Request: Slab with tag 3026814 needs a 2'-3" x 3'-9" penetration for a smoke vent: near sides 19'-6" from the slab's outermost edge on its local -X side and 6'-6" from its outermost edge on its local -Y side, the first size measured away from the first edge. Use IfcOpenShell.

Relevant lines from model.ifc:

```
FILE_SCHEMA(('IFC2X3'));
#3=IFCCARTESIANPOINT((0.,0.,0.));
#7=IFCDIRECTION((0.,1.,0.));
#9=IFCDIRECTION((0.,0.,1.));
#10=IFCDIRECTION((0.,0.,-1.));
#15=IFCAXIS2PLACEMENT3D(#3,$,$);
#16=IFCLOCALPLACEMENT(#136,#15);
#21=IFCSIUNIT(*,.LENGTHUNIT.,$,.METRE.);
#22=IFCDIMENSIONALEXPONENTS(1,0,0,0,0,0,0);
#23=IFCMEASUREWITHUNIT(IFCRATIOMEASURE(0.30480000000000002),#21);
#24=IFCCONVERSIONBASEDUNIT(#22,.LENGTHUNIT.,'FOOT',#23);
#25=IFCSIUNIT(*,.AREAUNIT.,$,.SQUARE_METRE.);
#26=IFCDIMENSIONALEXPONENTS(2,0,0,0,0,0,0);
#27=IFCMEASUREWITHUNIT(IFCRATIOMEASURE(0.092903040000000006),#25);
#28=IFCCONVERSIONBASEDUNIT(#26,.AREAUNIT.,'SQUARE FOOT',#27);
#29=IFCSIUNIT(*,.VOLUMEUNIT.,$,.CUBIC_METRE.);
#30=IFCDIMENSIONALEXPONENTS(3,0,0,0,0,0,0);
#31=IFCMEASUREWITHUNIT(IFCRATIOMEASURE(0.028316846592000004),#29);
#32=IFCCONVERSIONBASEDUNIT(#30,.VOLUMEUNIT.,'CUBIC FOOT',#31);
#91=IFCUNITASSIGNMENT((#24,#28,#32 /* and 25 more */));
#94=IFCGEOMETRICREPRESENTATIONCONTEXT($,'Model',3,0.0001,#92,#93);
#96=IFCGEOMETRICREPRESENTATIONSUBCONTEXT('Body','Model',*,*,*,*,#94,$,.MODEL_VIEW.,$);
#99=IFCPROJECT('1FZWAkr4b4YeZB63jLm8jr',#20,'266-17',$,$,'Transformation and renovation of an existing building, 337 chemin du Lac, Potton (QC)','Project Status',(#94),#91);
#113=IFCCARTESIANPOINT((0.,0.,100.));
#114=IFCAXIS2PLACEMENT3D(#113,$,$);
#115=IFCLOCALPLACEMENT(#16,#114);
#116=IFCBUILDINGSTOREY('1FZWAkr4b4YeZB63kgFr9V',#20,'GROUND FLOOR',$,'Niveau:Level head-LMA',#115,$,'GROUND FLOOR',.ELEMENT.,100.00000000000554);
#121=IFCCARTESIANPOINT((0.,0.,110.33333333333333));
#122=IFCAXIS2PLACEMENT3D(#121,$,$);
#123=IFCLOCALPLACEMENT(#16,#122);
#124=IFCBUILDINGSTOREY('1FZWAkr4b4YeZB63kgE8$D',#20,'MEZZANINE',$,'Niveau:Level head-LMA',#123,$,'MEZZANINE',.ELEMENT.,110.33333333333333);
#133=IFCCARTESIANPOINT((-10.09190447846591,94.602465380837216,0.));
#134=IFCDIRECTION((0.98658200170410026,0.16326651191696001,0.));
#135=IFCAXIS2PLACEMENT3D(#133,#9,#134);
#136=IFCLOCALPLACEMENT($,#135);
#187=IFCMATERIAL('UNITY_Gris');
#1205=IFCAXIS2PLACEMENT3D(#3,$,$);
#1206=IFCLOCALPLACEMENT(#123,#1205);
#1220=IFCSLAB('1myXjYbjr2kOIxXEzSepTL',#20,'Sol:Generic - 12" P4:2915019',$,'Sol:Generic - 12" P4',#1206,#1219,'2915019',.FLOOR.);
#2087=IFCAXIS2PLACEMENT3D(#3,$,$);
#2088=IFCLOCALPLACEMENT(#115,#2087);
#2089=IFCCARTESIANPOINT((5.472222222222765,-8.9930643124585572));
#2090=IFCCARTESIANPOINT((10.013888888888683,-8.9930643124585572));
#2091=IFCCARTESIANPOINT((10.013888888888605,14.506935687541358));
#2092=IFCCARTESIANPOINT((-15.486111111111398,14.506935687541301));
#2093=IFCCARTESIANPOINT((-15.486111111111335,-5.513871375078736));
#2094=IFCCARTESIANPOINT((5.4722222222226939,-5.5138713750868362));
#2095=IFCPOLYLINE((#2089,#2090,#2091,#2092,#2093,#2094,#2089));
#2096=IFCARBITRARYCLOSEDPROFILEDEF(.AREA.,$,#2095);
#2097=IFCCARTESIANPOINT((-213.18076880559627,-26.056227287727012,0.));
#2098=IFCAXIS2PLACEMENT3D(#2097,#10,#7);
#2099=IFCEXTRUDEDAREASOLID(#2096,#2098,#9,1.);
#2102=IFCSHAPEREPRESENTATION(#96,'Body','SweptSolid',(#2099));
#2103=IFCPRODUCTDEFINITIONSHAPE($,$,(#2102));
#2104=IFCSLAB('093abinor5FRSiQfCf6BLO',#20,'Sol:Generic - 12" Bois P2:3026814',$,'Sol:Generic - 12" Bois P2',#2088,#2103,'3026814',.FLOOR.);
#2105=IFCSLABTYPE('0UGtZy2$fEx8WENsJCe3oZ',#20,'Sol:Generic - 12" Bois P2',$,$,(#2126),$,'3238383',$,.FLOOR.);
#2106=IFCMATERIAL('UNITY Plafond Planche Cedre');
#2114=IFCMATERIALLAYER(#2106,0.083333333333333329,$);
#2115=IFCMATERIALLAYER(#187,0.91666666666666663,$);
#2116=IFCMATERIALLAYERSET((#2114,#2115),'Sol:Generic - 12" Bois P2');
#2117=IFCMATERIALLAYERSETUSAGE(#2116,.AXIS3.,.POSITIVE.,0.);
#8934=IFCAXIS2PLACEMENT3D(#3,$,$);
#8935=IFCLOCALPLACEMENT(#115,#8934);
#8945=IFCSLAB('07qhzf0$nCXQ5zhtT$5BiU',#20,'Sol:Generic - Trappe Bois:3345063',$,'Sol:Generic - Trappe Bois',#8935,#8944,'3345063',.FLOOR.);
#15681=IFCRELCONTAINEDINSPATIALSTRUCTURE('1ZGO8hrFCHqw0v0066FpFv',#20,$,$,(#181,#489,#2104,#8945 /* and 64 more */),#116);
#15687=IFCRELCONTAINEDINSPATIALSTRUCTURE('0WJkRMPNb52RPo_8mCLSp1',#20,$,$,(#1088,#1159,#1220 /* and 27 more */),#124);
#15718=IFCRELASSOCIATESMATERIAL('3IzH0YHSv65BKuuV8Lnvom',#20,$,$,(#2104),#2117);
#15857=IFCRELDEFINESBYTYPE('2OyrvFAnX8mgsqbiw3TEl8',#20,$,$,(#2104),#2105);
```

```python
import numpy as np
import ifcopenshell
import ifcopenshell.api.feature
import ifcopenshell.api.geometry
import ifcopenshell.api.root
import ifcopenshell.geom
import ifcopenshell.util.placement
import ifcopenshell.util.representation
import ifcopenshell.util.shape
import ifcopenshell.util.unit

model = ifcopenshell.open("model.ifc")
unit_scale = ifcopenshell.util.unit.calculate_unit_scale(model)
settings = ifcopenshell.geom.settings()


def volume(element):
    """Net volume in cubic metres, openings subtracted."""
    shape = ifcopenshell.geom.create_shape(settings, element)
    return ifcopenshell.util.shape.get_volume(shape.geometry)


slab = model.by_guid("093abinor5FRSiQfCf6BLO")
before = volume(slab)

# Extent in the slab's own axes, in metres. The edges named are its -X and -Y sides.
slab_shape = ifcopenshell.geom.create_shape(settings, slab)
vertices = ifcopenshell.util.shape.get_vertices(slab_shape.geometry)
x_min, y_min, bottom = vertices.min(axis=0)
top = vertices[:, 2].max()

opening = ifcopenshell.api.root.create_entity(model, ifc_class="IfcOpeningElement", name="Smoke vent opening")
context = ifcopenshell.util.representation.get_context(model, "Model", "Body", "MODEL_VIEW")
width, depth = 0.6858, 1.143
outline = [(0.0, 0.0), (width, 0.0), (width, depth), (0.0, depth), (0.0, 0.0)]
# Overshoot both faces by 50 mm so the cut is clean.
shape = ifcopenshell.api.geometry.add_slab_representation(
    model, context=context, depth=top - bottom + 0.1, polyline=outline
)
ifcopenshell.api.geometry.assign_representation(model, product=opening, representation=shape)

matrix = ifcopenshell.util.placement.get_local_placement(slab.ObjectPlacement)
matrix[:, 3] = matrix @ np.append(np.array([x_min + 5.9436, y_min + 1.9812, bottom - 0.05]) / unit_scale, 1.0)
ifcopenshell.api.geometry.edit_object_placement(model, product=opening, matrix=matrix, is_si=False)
ifcopenshell.api.feature.add_feature(model, feature=opening, element=slab)

after = volume(slab)

print(f"slab volume {before:.3f} -> {after:.3f} m3")

model.write("model_updated.ifc")
```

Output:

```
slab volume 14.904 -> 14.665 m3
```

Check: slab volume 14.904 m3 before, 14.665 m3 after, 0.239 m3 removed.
